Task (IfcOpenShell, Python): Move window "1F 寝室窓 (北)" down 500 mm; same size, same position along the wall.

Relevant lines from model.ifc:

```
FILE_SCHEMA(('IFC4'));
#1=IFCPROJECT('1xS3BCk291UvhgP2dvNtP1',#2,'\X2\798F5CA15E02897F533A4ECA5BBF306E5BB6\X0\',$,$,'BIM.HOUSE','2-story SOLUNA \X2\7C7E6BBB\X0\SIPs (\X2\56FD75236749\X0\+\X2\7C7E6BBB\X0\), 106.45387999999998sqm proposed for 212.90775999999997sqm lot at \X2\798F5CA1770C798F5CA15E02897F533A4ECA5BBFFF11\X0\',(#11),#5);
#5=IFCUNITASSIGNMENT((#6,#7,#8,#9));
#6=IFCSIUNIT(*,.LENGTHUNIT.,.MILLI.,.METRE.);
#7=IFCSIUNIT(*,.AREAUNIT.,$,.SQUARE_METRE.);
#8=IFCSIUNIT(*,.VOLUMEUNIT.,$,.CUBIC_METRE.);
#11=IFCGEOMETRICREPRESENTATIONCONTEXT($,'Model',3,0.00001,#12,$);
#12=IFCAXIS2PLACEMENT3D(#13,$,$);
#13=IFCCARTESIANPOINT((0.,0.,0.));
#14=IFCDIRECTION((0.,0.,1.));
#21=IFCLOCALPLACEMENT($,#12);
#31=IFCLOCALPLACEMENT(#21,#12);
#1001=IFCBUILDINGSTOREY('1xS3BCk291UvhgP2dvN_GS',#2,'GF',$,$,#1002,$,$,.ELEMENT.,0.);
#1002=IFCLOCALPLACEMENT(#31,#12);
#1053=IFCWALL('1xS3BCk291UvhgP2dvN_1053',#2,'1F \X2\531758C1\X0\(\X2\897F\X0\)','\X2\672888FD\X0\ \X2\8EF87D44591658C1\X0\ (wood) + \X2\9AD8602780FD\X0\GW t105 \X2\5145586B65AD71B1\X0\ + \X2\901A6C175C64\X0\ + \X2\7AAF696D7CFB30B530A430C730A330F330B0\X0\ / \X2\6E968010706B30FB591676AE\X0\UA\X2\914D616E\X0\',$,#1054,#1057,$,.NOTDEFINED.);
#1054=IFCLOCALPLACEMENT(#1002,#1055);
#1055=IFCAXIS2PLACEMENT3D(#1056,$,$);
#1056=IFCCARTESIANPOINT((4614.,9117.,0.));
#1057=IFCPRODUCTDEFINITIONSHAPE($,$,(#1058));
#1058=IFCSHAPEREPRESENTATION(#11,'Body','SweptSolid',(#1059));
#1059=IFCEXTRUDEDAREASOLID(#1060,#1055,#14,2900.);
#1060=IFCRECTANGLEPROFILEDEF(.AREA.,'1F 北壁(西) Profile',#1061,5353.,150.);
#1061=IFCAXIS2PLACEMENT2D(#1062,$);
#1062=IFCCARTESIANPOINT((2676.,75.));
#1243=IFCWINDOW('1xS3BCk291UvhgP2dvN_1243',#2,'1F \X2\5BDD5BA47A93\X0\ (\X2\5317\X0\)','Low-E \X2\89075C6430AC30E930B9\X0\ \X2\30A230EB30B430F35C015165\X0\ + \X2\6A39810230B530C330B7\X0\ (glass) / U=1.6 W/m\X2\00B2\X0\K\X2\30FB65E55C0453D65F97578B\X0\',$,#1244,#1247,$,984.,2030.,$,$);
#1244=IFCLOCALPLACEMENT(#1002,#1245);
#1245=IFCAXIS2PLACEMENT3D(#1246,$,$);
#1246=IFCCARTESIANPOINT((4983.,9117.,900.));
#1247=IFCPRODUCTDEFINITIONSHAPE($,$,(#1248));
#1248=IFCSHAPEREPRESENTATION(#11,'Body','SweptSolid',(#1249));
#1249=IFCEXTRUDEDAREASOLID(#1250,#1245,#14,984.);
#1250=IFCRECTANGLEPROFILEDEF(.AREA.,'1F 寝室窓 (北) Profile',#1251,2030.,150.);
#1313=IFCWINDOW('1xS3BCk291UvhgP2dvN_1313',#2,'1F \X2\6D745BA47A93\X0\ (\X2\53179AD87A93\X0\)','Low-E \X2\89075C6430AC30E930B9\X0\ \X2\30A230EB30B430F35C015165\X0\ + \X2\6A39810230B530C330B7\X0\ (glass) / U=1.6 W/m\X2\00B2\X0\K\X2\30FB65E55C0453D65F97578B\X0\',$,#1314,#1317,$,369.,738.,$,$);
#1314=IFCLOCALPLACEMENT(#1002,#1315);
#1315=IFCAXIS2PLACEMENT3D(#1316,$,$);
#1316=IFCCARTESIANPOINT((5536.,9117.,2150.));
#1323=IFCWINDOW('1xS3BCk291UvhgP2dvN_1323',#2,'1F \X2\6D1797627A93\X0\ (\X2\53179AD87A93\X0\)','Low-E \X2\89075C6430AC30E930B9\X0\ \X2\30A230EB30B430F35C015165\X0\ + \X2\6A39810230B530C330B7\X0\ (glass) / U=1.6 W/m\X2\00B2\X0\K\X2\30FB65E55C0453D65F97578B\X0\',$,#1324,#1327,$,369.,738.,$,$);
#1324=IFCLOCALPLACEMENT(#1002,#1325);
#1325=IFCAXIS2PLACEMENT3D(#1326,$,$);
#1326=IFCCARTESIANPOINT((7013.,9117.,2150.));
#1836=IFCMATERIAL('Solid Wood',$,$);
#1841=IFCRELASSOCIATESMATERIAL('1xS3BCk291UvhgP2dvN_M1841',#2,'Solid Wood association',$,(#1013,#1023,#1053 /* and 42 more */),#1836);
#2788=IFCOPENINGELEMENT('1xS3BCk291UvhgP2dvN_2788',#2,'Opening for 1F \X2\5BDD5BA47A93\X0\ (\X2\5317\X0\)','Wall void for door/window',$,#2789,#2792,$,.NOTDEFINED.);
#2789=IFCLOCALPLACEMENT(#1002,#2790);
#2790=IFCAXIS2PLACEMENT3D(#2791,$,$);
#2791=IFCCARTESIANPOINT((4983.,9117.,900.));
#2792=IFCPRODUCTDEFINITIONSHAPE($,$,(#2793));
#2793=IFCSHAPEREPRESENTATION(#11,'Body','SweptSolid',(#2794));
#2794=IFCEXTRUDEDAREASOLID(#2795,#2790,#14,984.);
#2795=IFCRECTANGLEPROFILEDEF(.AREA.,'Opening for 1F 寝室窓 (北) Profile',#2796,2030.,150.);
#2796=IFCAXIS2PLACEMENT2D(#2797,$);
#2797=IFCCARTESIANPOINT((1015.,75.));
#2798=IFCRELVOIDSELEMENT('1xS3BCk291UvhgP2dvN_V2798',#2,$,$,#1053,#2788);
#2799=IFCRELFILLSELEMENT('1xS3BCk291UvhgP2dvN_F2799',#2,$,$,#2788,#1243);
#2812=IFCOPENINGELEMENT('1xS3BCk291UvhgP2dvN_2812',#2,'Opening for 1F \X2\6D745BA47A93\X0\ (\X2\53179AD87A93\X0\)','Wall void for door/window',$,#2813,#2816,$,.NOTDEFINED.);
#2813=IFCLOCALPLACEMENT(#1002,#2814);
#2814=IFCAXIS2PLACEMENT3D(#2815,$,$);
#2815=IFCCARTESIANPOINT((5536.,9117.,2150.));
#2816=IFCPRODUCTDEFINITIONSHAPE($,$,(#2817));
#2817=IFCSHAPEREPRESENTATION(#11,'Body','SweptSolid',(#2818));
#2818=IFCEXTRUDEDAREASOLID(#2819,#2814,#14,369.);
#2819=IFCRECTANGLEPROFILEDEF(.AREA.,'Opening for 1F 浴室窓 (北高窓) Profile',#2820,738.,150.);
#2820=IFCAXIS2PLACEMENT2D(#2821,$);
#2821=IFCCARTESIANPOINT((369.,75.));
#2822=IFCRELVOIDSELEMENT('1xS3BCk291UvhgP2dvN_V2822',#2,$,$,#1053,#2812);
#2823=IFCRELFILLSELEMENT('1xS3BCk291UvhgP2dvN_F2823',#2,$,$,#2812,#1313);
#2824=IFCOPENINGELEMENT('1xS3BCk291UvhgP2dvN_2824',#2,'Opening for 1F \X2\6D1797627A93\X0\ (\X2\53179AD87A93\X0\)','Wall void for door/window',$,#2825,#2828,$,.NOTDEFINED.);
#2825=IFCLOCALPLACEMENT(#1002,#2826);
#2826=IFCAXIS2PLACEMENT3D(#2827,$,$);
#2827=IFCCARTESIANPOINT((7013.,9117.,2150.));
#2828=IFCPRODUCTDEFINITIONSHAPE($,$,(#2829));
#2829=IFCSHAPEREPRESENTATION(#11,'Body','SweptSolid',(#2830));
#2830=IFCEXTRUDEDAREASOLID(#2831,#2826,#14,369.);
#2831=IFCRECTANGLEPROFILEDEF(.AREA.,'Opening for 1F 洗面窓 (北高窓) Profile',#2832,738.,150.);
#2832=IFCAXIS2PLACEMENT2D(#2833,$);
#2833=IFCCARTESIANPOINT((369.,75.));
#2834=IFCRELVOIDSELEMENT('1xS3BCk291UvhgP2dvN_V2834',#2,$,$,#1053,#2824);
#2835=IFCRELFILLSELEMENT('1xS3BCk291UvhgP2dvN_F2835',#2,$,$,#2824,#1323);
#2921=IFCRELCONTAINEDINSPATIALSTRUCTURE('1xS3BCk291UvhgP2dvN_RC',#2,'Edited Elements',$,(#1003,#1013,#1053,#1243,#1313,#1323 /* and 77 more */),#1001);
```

```python
import numpy as np
import ifcopenshell
import ifcopenshell.api.geometry
import ifcopenshell.util.placement
import ifcopenshell.util.unit

model = ifcopenshell.open("model.ifc")
unit_scale = ifcopenshell.util.unit.calculate_unit_scale(model)

window = model.by_guid("1xS3BCk291UvhgP2dvN_1243")
opening = window.FillsVoids[0].RelatingOpeningElement
dz = -500.0

shift = np.array([0.0, 0.0, dz])
# The window is not placed relative to its opening, so move both.
for product in (opening, window):
    matrix = ifcopenshell.util.placement.get_local_placement(product.ObjectPlacement)
    matrix[:3, 3] += shift
    ifcopenshell.api.geometry.edit_object_placement(model, product=product, matrix=matrix, is_si=False)

print(f"moved by {dz * unit_scale:+.3f} m")

model.write("model-out.ifc")
```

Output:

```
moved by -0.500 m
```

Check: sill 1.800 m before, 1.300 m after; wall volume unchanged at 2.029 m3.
